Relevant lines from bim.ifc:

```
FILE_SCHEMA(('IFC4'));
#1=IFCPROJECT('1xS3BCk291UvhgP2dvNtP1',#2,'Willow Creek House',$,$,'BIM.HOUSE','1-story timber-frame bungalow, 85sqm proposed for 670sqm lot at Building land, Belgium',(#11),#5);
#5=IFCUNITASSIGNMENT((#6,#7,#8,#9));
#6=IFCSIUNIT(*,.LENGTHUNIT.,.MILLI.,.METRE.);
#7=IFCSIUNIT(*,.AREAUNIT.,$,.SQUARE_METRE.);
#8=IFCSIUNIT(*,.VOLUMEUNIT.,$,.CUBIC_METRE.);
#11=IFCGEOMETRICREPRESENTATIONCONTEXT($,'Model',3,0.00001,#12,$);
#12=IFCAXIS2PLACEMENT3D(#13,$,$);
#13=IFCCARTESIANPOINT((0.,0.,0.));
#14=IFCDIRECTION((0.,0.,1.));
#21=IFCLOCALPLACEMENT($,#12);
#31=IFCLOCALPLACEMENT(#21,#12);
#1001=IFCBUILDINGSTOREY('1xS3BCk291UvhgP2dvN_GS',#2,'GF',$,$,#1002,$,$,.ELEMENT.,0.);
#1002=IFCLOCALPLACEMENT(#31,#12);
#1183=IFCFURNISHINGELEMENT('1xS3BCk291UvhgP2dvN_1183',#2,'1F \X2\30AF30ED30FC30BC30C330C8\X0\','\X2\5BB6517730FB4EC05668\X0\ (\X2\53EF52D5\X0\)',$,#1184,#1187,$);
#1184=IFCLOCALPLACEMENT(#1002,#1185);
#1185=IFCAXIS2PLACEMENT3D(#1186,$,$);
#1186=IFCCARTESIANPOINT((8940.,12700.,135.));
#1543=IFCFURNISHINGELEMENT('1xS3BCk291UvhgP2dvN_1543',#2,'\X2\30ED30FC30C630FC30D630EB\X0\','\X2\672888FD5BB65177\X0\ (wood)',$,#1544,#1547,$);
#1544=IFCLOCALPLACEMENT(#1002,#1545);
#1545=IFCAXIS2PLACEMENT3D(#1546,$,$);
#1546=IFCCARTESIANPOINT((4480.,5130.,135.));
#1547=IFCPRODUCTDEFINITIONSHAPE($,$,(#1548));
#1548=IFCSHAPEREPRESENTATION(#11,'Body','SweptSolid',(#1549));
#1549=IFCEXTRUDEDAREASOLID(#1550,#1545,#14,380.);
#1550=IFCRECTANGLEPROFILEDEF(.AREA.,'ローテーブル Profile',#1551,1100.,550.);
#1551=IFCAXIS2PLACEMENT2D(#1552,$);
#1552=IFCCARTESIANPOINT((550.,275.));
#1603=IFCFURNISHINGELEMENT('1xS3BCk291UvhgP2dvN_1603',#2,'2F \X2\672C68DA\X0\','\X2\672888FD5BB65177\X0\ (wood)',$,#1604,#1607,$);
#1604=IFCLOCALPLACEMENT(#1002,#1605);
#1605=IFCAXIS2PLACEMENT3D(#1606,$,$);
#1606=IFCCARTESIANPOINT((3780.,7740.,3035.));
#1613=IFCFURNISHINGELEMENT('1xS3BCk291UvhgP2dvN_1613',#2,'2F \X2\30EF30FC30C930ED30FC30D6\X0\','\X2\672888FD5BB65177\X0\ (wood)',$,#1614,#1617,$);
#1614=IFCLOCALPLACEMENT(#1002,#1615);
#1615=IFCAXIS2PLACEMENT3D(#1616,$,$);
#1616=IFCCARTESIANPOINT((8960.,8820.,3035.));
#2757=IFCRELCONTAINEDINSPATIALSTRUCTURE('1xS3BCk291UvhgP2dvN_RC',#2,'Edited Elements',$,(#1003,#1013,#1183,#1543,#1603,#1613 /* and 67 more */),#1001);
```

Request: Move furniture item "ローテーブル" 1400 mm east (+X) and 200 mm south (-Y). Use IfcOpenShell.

```python
import ifcopenshell
import ifcopenshell.api.geometry
import ifcopenshell.util.placement

model = ifcopenshell.open("bim.ifc")

item = model.by_guid("1xS3BCk291UvhgP2dvN_1543")
matrix = ifcopenshell.util.placement.get_local_placement(item.ObjectPlacement)
matrix[0, 3] += 1400.0
matrix[1, 3] -= 200.0
ifcopenshell.api.geometry.edit_object_placement(model, product=item, matrix=matrix, is_si=False)

print(ifcopenshell.util.placement.get_local_placement(item.ObjectPlacement).round(3) + 0.0)

model.write("bim-out.ifc")
```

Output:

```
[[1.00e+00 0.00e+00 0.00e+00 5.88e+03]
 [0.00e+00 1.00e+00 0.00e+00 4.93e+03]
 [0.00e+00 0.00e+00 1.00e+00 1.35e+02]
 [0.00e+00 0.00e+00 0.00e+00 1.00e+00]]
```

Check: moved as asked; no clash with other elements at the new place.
